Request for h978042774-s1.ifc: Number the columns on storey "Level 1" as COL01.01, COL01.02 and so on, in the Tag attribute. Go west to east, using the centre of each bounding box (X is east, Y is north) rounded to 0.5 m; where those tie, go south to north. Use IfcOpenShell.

First a look at what the model holds.

```python
import ifcopenshell
import ifcopenshell.util.element
import ifcopenshell.util.placement

model = ifcopenshell.open("h978042774-s1.ifc")
print(model.schema)
storey = next(s for s in model.by_type("IfcBuildingStorey") if s.Name == "Level 1")
columns = [e for e in ifcopenshell.util.element.get_decomposition(storey) if e.is_a("IfcColumn")]
for e in sorted(columns, key=lambda e: e.id()):
    origin = ifcopenshell.util.placement.get_local_placement(e.ObjectPlacement)[:3, 3]
    print(e.id(), e.Tag, e.Name, origin.round(2) + 0.0, sep=" | ")
```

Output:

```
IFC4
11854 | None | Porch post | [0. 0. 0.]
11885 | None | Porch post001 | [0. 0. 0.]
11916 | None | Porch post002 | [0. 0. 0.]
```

```python
import ifcopenshell
import ifcopenshell.geom
import ifcopenshell.util.element
import ifcopenshell.util.shape

model = ifcopenshell.open("h978042774-s1.ifc")
settings = ifcopenshell.geom.settings()
settings.set("use-world-coords", True)


def centre(element):
    shape = ifcopenshell.geom.create_shape(settings, element)
    return ifcopenshell.util.shape.get_bbox_centroid(shape.geometry)


storey = next(s for s in model.by_type("IfcBuildingStorey") if s.Name == "Level 1")
columns = [e for e in ifcopenshell.util.element.get_decomposition(storey) if e.is_a("IfcColumn")]

# Insertion points can sit at a corner or the storey origin, so sort by the geometry (in metres).
centres = {e: centre(e) for e in columns}
columns.sort(key=lambda e: (round(centres[e][0] / 0.5), centres[e][1]))

for i, e in enumerate(columns, start=1):
    number = f"COL01.{i:02d}"
    e.Tag = number
    print(e.id(), number)

model.write("h978042774-s1-out.ifc")
```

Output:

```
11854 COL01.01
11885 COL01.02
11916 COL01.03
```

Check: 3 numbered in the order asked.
